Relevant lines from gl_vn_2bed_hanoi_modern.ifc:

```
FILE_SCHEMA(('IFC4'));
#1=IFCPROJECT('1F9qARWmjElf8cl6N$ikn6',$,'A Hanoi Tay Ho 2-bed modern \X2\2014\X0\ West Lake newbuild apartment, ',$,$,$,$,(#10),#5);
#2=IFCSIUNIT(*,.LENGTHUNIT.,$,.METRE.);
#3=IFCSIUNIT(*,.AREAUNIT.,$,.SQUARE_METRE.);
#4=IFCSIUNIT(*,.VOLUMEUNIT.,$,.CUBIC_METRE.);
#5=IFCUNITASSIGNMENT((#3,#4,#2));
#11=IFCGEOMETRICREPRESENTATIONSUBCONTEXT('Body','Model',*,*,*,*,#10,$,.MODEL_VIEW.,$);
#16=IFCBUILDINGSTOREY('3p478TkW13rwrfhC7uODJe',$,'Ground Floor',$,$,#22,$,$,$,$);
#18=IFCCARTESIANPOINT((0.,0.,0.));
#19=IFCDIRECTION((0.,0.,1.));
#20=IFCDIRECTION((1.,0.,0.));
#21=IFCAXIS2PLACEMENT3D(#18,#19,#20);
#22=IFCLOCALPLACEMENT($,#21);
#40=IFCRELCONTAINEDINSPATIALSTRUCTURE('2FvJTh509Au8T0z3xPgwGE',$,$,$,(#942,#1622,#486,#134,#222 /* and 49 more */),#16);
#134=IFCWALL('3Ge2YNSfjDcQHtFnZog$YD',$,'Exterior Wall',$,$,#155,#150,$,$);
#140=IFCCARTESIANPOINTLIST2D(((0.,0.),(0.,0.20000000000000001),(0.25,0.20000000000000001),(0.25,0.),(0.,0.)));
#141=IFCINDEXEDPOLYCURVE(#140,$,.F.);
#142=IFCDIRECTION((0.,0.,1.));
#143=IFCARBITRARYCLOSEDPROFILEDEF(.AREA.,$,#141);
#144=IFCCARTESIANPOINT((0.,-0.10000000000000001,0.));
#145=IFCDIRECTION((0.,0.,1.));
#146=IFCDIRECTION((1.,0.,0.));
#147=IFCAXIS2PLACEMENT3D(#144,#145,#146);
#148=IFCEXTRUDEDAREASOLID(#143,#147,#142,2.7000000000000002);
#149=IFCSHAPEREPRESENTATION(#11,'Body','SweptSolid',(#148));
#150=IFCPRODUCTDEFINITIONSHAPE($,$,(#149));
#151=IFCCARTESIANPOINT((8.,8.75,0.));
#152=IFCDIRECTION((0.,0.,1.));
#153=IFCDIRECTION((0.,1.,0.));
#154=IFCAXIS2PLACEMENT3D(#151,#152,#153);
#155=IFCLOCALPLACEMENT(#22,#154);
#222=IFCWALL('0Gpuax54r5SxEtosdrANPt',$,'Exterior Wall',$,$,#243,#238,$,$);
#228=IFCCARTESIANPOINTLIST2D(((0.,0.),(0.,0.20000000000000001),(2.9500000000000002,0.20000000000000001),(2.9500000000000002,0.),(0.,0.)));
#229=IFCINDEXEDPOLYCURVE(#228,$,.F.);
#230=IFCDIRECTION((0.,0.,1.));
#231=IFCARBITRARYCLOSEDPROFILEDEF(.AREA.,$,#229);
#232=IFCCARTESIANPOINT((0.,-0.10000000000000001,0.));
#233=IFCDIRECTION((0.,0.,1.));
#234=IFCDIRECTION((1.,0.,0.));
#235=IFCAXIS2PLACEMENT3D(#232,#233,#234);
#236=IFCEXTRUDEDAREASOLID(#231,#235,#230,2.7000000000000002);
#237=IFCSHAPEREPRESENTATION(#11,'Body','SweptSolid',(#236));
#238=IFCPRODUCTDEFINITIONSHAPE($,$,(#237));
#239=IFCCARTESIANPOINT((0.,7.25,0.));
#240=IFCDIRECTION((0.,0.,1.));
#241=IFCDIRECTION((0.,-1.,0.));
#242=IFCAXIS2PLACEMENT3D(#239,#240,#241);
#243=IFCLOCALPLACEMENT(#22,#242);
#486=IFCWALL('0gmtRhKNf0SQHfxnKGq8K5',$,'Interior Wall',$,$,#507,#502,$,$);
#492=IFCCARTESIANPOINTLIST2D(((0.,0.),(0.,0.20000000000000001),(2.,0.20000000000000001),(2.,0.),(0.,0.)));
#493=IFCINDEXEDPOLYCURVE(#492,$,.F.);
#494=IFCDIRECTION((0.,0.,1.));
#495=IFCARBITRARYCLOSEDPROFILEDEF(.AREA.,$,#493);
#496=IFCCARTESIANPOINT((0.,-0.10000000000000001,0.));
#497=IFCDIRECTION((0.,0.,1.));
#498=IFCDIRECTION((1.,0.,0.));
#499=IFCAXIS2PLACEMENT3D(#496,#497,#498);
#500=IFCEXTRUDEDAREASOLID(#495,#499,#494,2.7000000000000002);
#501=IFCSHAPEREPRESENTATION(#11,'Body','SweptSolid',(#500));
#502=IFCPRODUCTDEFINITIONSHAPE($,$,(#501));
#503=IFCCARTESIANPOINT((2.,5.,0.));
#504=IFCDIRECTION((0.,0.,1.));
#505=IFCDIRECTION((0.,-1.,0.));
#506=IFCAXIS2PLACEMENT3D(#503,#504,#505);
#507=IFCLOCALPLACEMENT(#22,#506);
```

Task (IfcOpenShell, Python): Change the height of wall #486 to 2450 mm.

```python
import ifcopenshell
import ifcopenshell.geom
import ifcopenshell.util.representation
import ifcopenshell.util.shape

model = ifcopenshell.open("gl_vn_2bed_hanoi_modern.ifc")
settings = ifcopenshell.geom.settings()


def volume(element):
    """Net volume in cubic metres, openings subtracted."""
    shape = ifcopenshell.geom.create_shape(settings, element)
    return ifcopenshell.util.shape.get_volume(shape.geometry)


wall = model.by_guid("0gmtRhKNf0SQHfxnKGq8K5")
before = volume(wall)

body = ifcopenshell.util.representation.get_representation(wall, "Model", "Body")
solid = body.Items[0]
old_height = solid.Depth
solid.Depth = 2.45
after = volume(wall)

print(f"height {old_height:g} -> {solid.Depth:g}, volume {before:.3f} -> {after:.3f} m3")

model.write("gl_vn_2bed_hanoi_modern_v2.ifc")
```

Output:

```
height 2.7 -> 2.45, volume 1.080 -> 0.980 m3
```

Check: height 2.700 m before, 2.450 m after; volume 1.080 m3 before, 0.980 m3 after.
